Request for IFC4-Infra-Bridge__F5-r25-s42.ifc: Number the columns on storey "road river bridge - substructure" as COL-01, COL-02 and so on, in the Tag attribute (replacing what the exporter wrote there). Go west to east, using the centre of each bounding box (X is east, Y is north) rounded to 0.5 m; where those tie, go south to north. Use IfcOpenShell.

First a look at what the model holds.

```python
import ifcopenshell
import ifcopenshell.util.element
import ifcopenshell.util.placement

model = ifcopenshell.open("IFC4-Infra-Bridge__F5-r25-s42.ifc")
print(model.schema)
storey = next(s for s in model.by_type("IfcBuildingStorey") if s.Name == "road river bridge - substructure")
columns = [e for e in ifcopenshell.util.element.get_decomposition(storey) if e.is_a("IfcColumn")]
for e in sorted(columns, key=lambda e: e.id()):
    origin = ifcopenshell.util.placement.get_local_placement(e.ObjectPlacement)[:3, 3]
    print(e.id(), e.Tag, e.Name, origin.round(2) + 0.0, sep=" | ")
```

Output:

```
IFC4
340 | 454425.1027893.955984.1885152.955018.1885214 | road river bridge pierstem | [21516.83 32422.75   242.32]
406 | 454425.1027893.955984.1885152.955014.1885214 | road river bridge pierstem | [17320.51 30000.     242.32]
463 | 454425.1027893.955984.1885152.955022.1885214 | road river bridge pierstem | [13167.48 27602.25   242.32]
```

```python
import ifcopenshell
import ifcopenshell.geom
import ifcopenshell.util.element
import ifcopenshell.util.shape

model = ifcopenshell.open("IFC4-Infra-Bridge__F5-r25-s42.ifc")
settings = ifcopenshell.geom.settings()
settings.set("use-world-coords", True)


def centre(element):
    shape = ifcopenshell.geom.create_shape(settings, element)
    return ifcopenshell.util.shape.get_bbox_centroid(shape.geometry)


storey = next(s for s in model.by_type("IfcBuildingStorey") if s.Name == "road river bridge - substructure")
columns = [e for e in ifcopenshell.util.element.get_decomposition(storey) if e.is_a("IfcColumn")]

# Insertion points can sit at a corner or the storey origin, so sort by the geometry (in metres).
centres = {e: centre(e) for e in columns}
columns.sort(key=lambda e: (round(centres[e][0] / 0.5), centres[e][1]))

for i, e in enumerate(columns, start=1):
    number = f"COL-{i:02d}"
    e.Tag = number
    print(e.id(), number)

model.write("IFC4-Infra-Bridge__F5-r25-s42_updated.ifc")
```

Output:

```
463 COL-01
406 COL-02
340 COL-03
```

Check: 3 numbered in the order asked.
